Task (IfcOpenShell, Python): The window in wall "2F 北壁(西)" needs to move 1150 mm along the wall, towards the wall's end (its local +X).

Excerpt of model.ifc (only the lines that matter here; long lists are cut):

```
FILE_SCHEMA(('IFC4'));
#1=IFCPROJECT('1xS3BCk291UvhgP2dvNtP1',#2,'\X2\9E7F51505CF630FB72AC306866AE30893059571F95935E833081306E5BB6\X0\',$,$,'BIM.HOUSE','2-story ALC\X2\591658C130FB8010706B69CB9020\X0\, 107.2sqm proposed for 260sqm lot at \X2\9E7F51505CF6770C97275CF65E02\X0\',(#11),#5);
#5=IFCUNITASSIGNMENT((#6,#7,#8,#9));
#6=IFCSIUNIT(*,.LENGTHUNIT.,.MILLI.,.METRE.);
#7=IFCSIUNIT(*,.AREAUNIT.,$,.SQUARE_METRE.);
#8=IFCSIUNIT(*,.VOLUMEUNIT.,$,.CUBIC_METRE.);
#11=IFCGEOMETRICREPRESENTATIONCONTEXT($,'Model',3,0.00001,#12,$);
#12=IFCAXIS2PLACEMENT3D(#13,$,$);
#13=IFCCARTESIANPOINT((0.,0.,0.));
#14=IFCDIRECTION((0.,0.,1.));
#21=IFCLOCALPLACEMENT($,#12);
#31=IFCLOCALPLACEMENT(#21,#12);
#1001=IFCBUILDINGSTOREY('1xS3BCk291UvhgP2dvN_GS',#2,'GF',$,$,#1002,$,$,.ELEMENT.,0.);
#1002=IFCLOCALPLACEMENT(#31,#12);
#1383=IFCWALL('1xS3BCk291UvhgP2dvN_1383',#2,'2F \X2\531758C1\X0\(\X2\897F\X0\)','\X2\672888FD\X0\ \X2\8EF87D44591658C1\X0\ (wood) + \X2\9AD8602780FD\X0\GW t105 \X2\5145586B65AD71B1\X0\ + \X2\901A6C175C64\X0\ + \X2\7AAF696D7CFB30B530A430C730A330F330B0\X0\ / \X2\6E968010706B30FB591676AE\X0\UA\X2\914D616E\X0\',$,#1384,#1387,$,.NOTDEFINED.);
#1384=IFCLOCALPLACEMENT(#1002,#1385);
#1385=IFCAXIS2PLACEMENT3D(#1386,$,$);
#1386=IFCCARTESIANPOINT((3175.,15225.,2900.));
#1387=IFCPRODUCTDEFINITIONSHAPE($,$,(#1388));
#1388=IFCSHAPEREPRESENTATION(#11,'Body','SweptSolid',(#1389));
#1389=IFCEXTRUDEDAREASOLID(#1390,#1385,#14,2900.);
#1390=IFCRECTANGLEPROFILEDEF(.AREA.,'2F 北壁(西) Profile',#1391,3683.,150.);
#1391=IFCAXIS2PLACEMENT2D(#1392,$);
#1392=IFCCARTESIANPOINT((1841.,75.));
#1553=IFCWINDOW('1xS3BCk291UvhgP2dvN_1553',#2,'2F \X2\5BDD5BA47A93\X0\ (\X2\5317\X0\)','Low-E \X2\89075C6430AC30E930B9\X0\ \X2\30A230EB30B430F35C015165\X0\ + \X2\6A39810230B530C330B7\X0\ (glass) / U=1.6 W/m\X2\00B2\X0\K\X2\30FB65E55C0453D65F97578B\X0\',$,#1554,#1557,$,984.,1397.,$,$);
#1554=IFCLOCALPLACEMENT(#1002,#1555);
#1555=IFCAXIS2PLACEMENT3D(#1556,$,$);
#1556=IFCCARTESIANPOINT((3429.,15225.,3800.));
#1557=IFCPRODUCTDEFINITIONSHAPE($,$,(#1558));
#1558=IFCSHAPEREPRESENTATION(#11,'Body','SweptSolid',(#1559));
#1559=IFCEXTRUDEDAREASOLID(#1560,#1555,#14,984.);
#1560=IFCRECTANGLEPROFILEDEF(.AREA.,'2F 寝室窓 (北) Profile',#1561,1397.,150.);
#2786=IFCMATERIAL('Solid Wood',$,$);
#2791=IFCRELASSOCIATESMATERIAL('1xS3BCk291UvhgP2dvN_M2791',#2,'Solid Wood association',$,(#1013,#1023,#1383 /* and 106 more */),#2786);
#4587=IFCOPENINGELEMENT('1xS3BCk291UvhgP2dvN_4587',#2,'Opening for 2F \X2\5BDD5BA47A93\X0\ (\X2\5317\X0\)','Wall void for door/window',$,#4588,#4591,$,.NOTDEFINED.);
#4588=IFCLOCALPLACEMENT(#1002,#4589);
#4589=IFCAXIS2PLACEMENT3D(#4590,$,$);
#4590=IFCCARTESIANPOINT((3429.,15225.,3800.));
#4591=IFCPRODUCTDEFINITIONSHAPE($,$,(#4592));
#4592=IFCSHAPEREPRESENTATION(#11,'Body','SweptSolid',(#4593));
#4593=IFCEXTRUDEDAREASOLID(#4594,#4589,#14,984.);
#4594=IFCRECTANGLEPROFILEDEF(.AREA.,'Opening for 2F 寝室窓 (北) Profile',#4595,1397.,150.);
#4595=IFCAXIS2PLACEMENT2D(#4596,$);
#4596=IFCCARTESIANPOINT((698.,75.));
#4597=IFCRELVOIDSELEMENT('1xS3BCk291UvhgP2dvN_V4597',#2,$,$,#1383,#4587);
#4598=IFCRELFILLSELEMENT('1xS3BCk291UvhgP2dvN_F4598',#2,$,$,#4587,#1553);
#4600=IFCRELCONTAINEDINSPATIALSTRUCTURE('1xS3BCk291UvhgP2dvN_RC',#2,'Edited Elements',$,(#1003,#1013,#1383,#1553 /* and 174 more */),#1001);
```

```python
import ifcopenshell
import ifcopenshell.api.geometry
import ifcopenshell.util.placement

model = ifcopenshell.open("model.ifc")

window = model.by_guid("1xS3BCk291UvhgP2dvN_1553")
opening = window.FillsVoids[0].RelatingOpeningElement
wall = opening.VoidsElements[0].RelatingBuildingElement

wall_matrix = ifcopenshell.util.placement.get_local_placement(wall.ObjectPlacement)
shift = wall_matrix[:3, 0] * 1150.0
before = ifcopenshell.util.placement.get_local_placement(window.ObjectPlacement)[:3, 3].copy()

# The window is not placed relative to its opening, so move both.
for product in (opening, window):
    matrix = ifcopenshell.util.placement.get_local_placement(product.ObjectPlacement)
    matrix[:3, 3] += shift
    ifcopenshell.api.geometry.edit_object_placement(model, product=product, matrix=matrix, is_si=False)

after = ifcopenshell.util.placement.get_local_placement(window.ObjectPlacement)[:3, 3]
print("window moved by", (after - before).round(3) + 0.0)

model.write("model_rev.ifc")
```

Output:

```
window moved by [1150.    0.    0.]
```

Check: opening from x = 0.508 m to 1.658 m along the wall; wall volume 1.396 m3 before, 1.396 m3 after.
